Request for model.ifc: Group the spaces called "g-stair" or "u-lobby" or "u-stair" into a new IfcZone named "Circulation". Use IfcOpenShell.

First a look at what the model holds.

```python
import ifcopenshell

model = ifcopenshell.open("model.ifc")
print(model.schema)
seen = {}
for space in model.by_type("IfcSpace"):
    seen[space.LongName] = seen.get(space.LongName, 0) + 1
for name, count in sorted(seen.items(), key=str):
    print(count, "x", name)
print("zones:", [z.Name for z in model.by_type("IfcZone")][:20])
```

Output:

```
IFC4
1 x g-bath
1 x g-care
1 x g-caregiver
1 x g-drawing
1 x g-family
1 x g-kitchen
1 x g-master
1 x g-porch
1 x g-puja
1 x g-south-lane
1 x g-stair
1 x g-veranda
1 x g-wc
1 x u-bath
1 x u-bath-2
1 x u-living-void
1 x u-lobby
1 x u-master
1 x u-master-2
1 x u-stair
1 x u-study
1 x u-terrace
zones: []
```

```python
import ifcopenshell
import ifcopenshell.api.group
import ifcopenshell.api.root

model = ifcopenshell.open("model.ifc")

names = {"g-stair", "u-lobby", "u-stair"}
spaces = [s for s in model.by_type("IfcSpace") if s.LongName in names]

zone = ifcopenshell.api.root.create_entity(model, ifc_class="IfcZone", name="Circulation")
ifcopenshell.api.group.assign_group(model, products=spaces, group=zone)
print(len(spaces), "spaces in", zone.Name)

model.write("model-out.ifc")
```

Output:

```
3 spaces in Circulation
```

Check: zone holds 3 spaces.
